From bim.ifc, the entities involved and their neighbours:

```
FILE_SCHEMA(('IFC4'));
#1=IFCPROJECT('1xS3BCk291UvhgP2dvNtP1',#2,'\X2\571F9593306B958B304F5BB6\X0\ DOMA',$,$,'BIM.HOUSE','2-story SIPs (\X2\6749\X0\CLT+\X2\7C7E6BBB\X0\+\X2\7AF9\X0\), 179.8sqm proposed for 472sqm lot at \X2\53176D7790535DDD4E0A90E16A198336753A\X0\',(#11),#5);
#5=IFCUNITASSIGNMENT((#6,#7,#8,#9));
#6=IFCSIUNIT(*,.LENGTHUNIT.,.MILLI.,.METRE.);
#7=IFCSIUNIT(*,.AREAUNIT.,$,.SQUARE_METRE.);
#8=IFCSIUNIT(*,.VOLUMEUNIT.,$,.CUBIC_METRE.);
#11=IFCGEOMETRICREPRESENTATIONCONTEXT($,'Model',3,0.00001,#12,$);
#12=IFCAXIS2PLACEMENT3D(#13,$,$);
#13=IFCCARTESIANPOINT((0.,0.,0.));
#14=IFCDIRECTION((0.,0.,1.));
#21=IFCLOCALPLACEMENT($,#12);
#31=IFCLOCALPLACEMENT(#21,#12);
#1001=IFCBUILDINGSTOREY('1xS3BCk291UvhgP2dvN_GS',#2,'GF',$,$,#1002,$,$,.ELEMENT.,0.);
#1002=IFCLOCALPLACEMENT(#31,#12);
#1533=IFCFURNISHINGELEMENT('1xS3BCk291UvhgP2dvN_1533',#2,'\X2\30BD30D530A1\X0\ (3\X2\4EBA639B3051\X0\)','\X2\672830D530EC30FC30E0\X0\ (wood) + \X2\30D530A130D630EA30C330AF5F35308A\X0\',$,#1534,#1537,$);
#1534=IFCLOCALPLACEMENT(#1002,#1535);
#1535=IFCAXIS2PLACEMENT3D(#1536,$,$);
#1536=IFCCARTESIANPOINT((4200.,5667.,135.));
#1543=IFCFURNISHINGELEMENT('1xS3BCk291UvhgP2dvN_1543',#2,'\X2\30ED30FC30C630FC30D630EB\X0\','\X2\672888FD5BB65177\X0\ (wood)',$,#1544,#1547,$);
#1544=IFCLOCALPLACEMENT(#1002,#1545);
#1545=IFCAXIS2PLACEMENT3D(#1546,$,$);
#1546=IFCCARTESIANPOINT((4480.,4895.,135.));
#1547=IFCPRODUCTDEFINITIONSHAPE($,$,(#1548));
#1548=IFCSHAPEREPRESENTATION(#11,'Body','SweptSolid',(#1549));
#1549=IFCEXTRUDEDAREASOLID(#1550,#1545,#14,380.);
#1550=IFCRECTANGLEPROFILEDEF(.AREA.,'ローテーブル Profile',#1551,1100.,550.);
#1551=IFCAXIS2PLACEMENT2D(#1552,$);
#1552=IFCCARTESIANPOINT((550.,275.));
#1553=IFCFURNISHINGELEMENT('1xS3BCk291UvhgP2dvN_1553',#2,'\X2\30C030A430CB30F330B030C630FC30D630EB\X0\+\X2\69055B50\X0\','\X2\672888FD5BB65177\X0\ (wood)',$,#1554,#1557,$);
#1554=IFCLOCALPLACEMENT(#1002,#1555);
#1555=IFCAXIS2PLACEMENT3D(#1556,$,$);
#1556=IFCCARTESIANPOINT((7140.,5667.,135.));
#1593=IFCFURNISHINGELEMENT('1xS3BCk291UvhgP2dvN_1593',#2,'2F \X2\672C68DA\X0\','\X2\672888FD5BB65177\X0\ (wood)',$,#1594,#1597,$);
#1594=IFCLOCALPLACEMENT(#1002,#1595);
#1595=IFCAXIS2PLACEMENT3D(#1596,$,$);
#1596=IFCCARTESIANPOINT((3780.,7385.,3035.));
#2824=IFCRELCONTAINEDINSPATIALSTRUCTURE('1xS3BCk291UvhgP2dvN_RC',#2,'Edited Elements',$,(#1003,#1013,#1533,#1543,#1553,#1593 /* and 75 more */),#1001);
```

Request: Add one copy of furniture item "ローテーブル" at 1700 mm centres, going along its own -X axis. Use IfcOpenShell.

```python
import ifcopenshell
import ifcopenshell.api.geometry
import ifcopenshell.api.root
import ifcopenshell.util.element
import ifcopenshell.util.placement

model = ifcopenshell.open("bim.ifc")


def reuse_history(source, copy):
    """copy_class also copies each property set's owner history, people and application; keep the originals."""
    for rel in copy.IsDefinedBy:
        if rel.is_a("IfcRelDefinesByProperties") and (history := rel.RelatingPropertyDefinition.OwnerHistory):
            rel.RelatingPropertyDefinition.OwnerHistory = source.OwnerHistory
            ifcopenshell.util.element.remove_deep2(model, history)


source = model.by_guid("1xS3BCk291UvhgP2dvN_1543")
base = ifcopenshell.util.placement.get_local_placement(source.ObjectPlacement)
step = -base[:3, 0] * 1700.0

for i in range(1, 2):
    copy = ifcopenshell.api.root.copy_class(model, product=source)
    copy.Representation = ifcopenshell.util.element.copy_deep(
        model, source.Representation, exclude=["IfcGeometricRepresentationContext", "IfcRepresentationMap"]
    )
    reuse_history(source, copy)
    matrix = base.copy()
    matrix[:3, 3] += i * step
    print("added at", matrix[:3, 3].round(3) + 0.0)
    ifcopenshell.api.geometry.edit_object_placement(model, product=copy, matrix=matrix, is_si=False)

model.write("bim_updated.ifc")
```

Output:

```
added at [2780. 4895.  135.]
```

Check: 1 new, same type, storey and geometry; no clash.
